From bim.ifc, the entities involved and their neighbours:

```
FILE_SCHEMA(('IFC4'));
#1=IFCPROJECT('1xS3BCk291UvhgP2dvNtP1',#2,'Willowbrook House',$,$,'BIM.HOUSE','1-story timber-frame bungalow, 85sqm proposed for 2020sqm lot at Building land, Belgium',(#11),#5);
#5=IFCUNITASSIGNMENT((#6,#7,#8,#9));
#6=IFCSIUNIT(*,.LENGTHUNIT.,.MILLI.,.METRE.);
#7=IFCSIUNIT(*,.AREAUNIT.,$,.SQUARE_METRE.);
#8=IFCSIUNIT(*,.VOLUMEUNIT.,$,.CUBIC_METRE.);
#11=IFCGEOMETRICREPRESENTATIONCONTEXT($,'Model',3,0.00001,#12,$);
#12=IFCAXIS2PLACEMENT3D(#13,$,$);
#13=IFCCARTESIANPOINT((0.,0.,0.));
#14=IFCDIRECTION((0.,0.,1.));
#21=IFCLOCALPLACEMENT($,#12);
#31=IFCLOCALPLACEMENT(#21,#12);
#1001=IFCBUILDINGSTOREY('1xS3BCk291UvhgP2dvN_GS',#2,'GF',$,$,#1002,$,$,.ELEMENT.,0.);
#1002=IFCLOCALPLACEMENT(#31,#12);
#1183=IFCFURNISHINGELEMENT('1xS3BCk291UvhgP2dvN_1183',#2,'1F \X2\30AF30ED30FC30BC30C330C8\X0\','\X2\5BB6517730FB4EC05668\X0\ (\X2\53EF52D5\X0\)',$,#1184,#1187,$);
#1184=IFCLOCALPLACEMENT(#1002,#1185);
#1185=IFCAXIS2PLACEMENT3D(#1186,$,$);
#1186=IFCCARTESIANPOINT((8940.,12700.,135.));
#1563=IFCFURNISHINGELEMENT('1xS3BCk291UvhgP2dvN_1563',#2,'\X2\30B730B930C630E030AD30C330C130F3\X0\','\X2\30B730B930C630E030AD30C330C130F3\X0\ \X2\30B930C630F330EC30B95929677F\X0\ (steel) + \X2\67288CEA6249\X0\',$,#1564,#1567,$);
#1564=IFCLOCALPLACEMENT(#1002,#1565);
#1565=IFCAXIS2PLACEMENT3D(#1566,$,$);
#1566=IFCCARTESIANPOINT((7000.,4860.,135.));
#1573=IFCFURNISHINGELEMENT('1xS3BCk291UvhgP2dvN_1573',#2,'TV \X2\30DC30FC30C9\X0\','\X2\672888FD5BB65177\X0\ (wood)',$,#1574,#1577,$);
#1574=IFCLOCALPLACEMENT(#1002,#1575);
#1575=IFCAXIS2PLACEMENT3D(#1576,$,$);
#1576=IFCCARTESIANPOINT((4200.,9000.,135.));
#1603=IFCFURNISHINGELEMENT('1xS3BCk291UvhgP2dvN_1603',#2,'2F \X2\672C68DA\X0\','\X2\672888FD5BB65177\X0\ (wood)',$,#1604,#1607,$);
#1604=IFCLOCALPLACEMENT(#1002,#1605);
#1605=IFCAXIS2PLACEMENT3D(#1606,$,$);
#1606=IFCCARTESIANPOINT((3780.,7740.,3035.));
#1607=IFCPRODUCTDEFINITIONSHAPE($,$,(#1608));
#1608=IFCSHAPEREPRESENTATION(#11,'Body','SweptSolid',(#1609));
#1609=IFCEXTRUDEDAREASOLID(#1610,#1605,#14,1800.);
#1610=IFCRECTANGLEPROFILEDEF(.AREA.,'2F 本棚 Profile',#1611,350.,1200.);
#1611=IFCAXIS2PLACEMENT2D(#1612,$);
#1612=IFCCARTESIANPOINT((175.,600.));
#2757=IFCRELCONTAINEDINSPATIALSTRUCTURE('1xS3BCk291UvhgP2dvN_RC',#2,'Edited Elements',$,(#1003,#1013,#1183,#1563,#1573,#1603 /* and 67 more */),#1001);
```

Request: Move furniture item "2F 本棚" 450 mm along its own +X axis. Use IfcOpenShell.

```python
import ifcopenshell
import ifcopenshell.api.geometry
import ifcopenshell.util.placement
import ifcopenshell.util.unit

model = ifcopenshell.open("bim.ifc")
unit_scale = ifcopenshell.util.unit.calculate_unit_scale(model)

item = model.by_guid("1xS3BCk291UvhgP2dvN_1603")
matrix = ifcopenshell.util.placement.get_local_placement(item.ObjectPlacement)
matrix[:3, 3] += matrix[:3, 0] * 0.45 / unit_scale
ifcopenshell.api.geometry.edit_object_placement(model, product=item, matrix=matrix, is_si=False)

print(ifcopenshell.util.placement.get_local_placement(item.ObjectPlacement).round(3) + 0.0)

model.write("bim_edited.ifc")
```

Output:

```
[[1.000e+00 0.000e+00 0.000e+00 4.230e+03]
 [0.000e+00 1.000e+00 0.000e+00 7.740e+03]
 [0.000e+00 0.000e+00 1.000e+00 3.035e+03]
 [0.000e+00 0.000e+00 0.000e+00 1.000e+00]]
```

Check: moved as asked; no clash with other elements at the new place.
